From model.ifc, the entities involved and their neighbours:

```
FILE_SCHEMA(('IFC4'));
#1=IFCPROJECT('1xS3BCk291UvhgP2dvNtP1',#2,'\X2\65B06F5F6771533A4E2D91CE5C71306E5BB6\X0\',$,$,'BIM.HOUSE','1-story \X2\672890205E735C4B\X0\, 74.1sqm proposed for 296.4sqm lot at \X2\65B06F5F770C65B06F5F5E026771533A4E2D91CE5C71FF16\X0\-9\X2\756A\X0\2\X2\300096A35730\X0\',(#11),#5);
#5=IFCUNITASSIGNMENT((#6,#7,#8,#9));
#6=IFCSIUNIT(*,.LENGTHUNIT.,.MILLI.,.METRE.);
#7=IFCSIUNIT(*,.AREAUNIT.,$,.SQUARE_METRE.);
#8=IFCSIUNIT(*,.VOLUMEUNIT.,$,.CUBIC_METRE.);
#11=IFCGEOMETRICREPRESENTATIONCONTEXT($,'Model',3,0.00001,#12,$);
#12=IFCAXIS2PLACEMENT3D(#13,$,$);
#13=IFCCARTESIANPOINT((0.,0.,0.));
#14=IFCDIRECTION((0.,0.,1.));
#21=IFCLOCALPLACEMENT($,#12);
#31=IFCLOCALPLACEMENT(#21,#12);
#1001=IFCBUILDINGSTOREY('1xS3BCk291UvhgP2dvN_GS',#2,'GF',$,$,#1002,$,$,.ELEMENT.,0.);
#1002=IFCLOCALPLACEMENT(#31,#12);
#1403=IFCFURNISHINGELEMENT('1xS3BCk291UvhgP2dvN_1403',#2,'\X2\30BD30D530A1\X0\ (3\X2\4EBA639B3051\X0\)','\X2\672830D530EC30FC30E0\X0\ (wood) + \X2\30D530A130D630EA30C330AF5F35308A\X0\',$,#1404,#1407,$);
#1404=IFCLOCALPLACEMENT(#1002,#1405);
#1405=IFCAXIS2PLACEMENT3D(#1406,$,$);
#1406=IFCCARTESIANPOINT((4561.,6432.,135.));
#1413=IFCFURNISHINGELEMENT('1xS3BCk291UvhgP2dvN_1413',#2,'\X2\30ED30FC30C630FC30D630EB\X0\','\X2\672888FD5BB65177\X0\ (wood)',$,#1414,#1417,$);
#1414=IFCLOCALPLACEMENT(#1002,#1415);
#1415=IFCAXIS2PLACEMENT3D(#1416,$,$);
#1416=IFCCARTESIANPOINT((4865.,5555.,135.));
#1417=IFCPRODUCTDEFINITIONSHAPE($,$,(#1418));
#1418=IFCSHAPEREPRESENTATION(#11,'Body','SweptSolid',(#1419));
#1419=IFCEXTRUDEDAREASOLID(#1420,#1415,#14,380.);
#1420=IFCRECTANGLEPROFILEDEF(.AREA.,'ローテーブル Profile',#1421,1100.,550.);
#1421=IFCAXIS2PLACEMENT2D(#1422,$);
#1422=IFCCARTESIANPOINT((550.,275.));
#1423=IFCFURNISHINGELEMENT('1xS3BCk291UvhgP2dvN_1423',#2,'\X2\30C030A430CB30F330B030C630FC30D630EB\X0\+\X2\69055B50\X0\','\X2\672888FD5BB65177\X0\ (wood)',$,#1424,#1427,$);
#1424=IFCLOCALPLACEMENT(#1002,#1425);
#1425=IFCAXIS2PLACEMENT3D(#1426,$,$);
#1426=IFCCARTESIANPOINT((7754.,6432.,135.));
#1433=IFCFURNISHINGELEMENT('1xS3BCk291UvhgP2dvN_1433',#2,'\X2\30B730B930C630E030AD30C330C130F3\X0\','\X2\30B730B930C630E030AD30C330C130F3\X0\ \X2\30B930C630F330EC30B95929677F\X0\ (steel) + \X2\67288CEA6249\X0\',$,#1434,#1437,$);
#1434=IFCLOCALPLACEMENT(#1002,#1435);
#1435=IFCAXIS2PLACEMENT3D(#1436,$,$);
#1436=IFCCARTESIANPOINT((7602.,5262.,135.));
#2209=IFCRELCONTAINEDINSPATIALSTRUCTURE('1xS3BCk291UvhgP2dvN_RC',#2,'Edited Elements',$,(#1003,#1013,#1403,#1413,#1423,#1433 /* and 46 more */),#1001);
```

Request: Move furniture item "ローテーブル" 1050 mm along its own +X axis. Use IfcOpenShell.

```python
import ifcopenshell
import ifcopenshell.api.geometry
import ifcopenshell.util.placement
import ifcopenshell.util.unit

model = ifcopenshell.open("model.ifc")
unit_scale = ifcopenshell.util.unit.calculate_unit_scale(model)

item = model.by_guid("1xS3BCk291UvhgP2dvN_1413")
matrix = ifcopenshell.util.placement.get_local_placement(item.ObjectPlacement)
matrix[:3, 3] += matrix[:3, 0] * 1.05 / unit_scale
ifcopenshell.api.geometry.edit_object_placement(model, product=item, matrix=matrix, is_si=False)

print(ifcopenshell.util.placement.get_local_placement(item.ObjectPlacement).round(3) + 0.0)

model.write("model-out.ifc")
```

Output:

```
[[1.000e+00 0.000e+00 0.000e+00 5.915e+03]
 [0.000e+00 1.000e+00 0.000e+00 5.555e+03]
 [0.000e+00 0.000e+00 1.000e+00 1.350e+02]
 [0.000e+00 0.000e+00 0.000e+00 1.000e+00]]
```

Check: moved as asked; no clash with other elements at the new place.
